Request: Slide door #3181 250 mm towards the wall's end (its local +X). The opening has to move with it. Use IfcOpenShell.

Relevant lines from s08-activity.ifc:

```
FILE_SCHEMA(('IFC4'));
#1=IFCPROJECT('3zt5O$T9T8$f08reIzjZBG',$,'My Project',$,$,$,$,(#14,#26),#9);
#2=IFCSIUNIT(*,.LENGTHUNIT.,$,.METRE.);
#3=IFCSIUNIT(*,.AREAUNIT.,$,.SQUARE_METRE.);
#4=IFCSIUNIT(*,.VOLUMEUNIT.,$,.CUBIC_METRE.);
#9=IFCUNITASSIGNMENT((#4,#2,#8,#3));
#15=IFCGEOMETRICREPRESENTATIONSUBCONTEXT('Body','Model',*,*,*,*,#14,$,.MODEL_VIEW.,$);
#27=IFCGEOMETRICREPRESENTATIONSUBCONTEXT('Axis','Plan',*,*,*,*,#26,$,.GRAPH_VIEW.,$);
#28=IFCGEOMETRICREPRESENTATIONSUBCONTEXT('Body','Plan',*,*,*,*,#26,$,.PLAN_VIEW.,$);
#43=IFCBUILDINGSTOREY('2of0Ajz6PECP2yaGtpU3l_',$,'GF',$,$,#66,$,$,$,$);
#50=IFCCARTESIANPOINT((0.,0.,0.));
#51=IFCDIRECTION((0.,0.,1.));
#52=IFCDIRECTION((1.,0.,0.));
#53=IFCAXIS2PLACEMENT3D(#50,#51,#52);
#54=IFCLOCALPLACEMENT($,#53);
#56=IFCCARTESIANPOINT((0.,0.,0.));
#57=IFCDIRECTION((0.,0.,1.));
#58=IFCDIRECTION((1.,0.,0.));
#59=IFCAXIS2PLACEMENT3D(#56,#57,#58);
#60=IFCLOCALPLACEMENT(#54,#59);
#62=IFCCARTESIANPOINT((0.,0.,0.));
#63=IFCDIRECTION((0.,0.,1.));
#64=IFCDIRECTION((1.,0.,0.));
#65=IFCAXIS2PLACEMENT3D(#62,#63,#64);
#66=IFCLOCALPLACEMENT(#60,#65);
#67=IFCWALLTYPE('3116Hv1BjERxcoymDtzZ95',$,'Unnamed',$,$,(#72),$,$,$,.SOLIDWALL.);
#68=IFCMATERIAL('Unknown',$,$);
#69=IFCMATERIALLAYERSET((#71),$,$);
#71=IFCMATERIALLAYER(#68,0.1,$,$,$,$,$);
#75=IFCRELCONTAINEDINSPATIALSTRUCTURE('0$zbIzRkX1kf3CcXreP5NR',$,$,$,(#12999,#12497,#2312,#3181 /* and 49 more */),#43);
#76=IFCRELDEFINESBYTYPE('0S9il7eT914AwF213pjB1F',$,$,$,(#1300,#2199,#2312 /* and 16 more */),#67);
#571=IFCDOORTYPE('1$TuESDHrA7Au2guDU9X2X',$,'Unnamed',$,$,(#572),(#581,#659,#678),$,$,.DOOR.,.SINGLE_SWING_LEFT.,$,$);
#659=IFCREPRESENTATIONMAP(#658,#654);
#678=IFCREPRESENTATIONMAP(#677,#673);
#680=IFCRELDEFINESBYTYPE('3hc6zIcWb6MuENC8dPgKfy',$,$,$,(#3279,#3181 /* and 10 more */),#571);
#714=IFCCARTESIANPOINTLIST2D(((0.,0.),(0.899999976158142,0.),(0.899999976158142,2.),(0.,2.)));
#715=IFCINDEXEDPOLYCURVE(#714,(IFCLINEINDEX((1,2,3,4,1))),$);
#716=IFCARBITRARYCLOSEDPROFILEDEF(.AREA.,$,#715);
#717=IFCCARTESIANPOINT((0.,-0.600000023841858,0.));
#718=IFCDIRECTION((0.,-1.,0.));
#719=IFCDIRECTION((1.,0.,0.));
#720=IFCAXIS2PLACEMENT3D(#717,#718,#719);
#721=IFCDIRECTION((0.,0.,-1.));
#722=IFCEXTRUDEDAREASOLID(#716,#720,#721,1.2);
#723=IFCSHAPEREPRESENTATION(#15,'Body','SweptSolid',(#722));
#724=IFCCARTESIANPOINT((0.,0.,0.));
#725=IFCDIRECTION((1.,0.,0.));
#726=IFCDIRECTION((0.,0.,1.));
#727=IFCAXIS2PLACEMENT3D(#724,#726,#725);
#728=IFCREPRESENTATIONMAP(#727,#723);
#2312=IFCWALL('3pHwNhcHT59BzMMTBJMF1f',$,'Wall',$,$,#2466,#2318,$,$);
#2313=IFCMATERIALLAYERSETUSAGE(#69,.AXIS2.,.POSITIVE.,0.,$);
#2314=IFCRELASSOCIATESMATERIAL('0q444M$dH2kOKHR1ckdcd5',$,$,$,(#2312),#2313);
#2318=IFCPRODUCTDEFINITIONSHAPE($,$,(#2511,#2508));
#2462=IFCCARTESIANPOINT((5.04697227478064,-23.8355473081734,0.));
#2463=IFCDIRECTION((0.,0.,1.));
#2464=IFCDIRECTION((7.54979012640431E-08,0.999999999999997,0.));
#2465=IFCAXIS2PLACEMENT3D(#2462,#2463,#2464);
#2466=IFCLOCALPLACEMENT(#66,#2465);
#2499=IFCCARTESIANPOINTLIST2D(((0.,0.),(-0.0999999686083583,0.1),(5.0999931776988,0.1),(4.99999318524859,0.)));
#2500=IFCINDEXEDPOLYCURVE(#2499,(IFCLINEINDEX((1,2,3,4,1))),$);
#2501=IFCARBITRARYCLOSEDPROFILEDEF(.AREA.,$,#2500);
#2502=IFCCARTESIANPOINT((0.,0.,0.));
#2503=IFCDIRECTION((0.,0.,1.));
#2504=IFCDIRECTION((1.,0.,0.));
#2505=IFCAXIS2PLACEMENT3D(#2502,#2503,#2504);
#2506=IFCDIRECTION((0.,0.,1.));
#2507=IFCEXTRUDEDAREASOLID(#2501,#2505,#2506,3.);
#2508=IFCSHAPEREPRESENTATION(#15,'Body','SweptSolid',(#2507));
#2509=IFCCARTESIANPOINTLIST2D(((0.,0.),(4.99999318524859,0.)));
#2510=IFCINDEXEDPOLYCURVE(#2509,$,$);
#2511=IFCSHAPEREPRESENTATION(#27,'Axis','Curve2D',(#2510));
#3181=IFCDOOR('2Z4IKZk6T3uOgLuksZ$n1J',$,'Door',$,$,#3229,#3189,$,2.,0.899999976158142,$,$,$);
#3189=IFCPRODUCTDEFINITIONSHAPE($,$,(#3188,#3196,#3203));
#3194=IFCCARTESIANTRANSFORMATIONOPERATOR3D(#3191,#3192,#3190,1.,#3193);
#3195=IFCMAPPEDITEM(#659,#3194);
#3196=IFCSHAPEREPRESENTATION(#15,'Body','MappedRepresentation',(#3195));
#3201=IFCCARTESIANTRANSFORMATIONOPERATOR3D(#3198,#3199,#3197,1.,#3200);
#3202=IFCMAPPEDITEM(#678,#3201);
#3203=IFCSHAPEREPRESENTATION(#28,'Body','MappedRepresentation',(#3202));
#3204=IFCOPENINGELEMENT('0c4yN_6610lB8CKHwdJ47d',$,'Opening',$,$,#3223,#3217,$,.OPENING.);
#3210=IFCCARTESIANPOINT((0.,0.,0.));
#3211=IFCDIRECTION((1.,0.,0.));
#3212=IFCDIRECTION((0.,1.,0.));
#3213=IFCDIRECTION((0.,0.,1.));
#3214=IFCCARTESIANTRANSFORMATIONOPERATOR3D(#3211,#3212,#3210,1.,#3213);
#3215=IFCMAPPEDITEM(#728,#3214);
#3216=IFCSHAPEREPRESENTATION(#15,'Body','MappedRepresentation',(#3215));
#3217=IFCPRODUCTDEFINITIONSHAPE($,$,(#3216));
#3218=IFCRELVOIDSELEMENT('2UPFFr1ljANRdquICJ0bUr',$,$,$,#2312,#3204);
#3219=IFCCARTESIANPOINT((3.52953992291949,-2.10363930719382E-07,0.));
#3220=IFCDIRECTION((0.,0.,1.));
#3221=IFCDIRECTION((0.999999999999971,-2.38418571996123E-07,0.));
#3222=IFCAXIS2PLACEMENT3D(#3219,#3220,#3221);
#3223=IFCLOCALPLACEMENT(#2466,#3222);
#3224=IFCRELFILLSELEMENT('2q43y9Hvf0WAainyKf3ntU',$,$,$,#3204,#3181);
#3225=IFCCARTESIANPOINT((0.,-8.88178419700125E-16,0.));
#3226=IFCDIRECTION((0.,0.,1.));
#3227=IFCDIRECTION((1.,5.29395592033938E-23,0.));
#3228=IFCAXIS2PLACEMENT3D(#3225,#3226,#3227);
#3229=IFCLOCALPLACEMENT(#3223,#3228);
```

```python
import ifcopenshell
import ifcopenshell.api.geometry
import ifcopenshell.util.placement
import ifcopenshell.util.unit

model = ifcopenshell.open("s08-activity.ifc")
unit_scale = ifcopenshell.util.unit.calculate_unit_scale(model)

door = model.by_guid("2Z4IKZk6T3uOgLuksZ$n1J")
opening = door.FillsVoids[0].RelatingOpeningElement
wall = opening.VoidsElements[0].RelatingBuildingElement

wall_matrix = ifcopenshell.util.placement.get_local_placement(wall.ObjectPlacement)
shift = wall_matrix[:3, 0] * 0.25 / unit_scale
before = ifcopenshell.util.placement.get_local_placement(door.ObjectPlacement)[:3, 3].copy()

# The door is placed relative to its opening, so it follows when the opening moves.
matrix = ifcopenshell.util.placement.get_local_placement(opening.ObjectPlacement)
matrix[:3, 3] += shift
ifcopenshell.api.geometry.edit_object_placement(
    model, product=opening, matrix=matrix, is_si=False, should_transform_children=True
)

after = ifcopenshell.util.placement.get_local_placement(door.ObjectPlacement)[:3, 3]
print("door moved by", (after - before).round(3) + 0.0)

model.write("s08-activity_edited.ifc")
```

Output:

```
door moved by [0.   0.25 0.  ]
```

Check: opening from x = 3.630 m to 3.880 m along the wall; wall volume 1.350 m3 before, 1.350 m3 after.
